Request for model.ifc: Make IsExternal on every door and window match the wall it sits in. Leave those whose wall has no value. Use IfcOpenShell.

First a look at what the model holds.

```python
import ifcopenshell
import ifcopenshell.util.element

model = ifcopenshell.open("model.ifc")
print(model.schema)
seen = {}
for e in model.by_type("IfcDoor") + model.by_type("IfcWindow"):
    if not e.FillsVoids:
        continue
    host = e.FillsVoids[0].RelatingOpeningElement.VoidsElements[0].RelatingBuildingElement
    own = ifcopenshell.util.element.get_pset(e, f"Pset_{e.is_a()[3:].removesuffix('StandardCase')}Common", "IsExternal")
    wall = ifcopenshell.util.element.get_pset(host, "Pset_WallCommon", "IsExternal")
    seen[e.is_a(), own, wall] = seen.get((e.is_a(), own, wall), 0) + 1
for (cls, own, wall), count in sorted(seen.items(), key=str):
    print(count, cls, "IsExternal:", own, "| host wall:", wall)
```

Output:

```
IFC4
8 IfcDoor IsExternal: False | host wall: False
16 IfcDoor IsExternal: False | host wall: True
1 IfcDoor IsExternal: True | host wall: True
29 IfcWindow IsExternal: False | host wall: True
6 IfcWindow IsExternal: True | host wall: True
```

```python
import ifcopenshell
import ifcopenshell.api.pset
import ifcopenshell.util.element

model = ifcopenshell.open("model.ifc")

count = 0
for ifc_class, pset_name in (("IfcDoor", "Pset_DoorCommon"), ("IfcWindow", "Pset_WindowCommon")):
    for e in model.by_type(ifc_class):
        if not e.FillsVoids:
            continue
        host = e.FillsVoids[0].RelatingOpeningElement.VoidsElements[0].RelatingBuildingElement
        external = ifcopenshell.util.element.get_pset(host, "Pset_WallCommon", "IsExternal")
        if external is None or ifcopenshell.util.element.get_pset(e, pset_name, "IsExternal") == external:
            continue
        pset = ifcopenshell.api.pset.add_pset(model, product=e, name=pset_name)
        ifcopenshell.api.pset.edit_pset(model, pset=pset, properties={"IsExternal": external})
        count += 1

print(count, "updated")

model.write("model_rev.ifc")
```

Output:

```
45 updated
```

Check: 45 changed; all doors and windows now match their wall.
